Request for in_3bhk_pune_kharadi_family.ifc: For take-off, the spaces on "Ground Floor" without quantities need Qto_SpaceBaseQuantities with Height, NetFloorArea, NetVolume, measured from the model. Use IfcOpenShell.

First a look at what the model holds.

```python
import ifcopenshell
import ifcopenshell.util.element
import ifcopenshell.util.unit

model = ifcopenshell.open("in_3bhk_pune_kharadi_family.ifc")
print(model.schema)
for unit_type in ("LENGTHUNIT", "AREAUNIT", "VOLUMEUNIT"):
    print(unit_type, ifcopenshell.util.unit.calculate_unit_scale(model, unit_type))
storey = next(s for s in model.by_type("IfcBuildingStorey") if s.Name == "Ground Floor")
spaces = [e for e in ifcopenshell.util.element.get_decomposition(storey) if e.is_a("IfcSpace")]
for e in sorted(spaces, key=lambda e: e.id()):
    print(e.id(), e.is_a(), e.Name, list(ifcopenshell.util.element.get_psets(e, qtos_only=True)), sep=" | ")
```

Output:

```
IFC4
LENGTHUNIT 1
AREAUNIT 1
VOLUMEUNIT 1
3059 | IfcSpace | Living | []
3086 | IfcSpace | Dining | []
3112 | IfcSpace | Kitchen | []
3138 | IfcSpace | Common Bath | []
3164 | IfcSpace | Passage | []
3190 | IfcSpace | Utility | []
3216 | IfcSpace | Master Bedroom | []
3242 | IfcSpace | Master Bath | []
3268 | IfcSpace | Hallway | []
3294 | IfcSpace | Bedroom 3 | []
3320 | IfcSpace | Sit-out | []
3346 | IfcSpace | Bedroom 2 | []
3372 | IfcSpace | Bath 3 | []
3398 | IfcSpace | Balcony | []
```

```python
import ifcopenshell
import ifcopenshell.api.pset
import ifcopenshell.geom
import ifcopenshell.util.element
import ifcopenshell.util.shape
import ifcopenshell.util.unit

model = ifcopenshell.open("in_3bhk_pune_kharadi_family.ifc")
unit_scale = ifcopenshell.util.unit.calculate_unit_scale(model)
area_scale = ifcopenshell.util.unit.calculate_unit_scale(model, "AREAUNIT")
volume_scale = ifcopenshell.util.unit.calculate_unit_scale(model, "VOLUMEUNIT")
settings = ifcopenshell.geom.settings()

storey = next(s for s in model.by_type("IfcBuildingStorey") if s.Name == "Ground Floor")
spaces = [e for e in ifcopenshell.util.element.get_decomposition(storey) if e.is_a("IfcSpace")]

for e in sorted(spaces, key=lambda e: e.id()):
    if ifcopenshell.util.element.get_psets(e, qtos_only=True, should_inherit=False):
        continue
    # Geometry comes back in metres, in the element's own axes.
    shape = ifcopenshell.geom.create_shape(settings, e)
    values = {
        "Height": ifcopenshell.util.shape.get_z(shape.geometry) / unit_scale,
        "NetFloorArea": ifcopenshell.util.shape.get_footprint_area(shape.geometry) / area_scale,
        "NetVolume": ifcopenshell.util.shape.get_volume(shape.geometry) / volume_scale,
    }
    qto = ifcopenshell.api.pset.add_qto(model, product=e, name="Qto_SpaceBaseQuantities")
    ifcopenshell.api.pset.edit_qto(model, qto=qto, properties=values)
    print(e.id(), {k: round(v, 3) for k, v in values.items()})

model.write("in_3bhk_pune_kharadi_family_rev.ifc")
```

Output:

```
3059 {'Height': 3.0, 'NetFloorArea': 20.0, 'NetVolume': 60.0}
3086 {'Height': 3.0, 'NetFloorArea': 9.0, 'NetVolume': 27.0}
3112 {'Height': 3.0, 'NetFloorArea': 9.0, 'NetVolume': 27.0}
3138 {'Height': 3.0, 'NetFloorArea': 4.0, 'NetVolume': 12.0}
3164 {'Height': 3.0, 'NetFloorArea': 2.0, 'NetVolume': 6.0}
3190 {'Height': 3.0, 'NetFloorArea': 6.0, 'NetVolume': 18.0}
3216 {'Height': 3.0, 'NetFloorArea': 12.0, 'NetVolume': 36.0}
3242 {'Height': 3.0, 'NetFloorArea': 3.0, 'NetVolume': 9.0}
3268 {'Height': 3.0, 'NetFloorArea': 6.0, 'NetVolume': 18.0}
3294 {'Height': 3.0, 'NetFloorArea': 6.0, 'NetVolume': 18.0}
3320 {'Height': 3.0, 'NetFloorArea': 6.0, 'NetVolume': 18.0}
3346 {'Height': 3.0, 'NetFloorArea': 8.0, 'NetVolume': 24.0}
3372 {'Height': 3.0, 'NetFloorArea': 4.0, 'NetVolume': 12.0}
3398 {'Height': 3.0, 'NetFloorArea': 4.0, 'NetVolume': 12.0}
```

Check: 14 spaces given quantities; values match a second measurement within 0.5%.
